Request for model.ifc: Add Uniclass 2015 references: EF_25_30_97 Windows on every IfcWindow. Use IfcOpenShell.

First a look at what the model holds.

```python
import ifcopenshell

model = ifcopenshell.open("model.ifc")
print(model.schema)
print("classifications:", [c.Name for c in model.by_type("IfcClassification")])
for ifc_class in ("IfcDoor", "IfcRoof", "IfcStair", "IfcWall", "IfcWindow"):
    print(ifc_class, len(model.by_type(ifc_class)))
```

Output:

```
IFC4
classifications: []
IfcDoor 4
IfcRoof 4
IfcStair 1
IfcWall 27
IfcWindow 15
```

```python
import ifcopenshell
import ifcopenshell.api.classification

model = ifcopenshell.open("model.ifc")

system = ifcopenshell.api.classification.add_classification(model, classification="Uniclass 2015")

codes = {
    "IfcWindow": ("EF_25_30_97", "Windows"),
}
for ifc_class, (code, name) in codes.items():
    products = model.by_type(ifc_class)
    ifcopenshell.api.classification.add_reference(
        model, products=products, classification=system, identification=code, name=name
    )
    print(code, len(products))

model.write("model_rev.ifc")
```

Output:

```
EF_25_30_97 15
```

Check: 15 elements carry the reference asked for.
